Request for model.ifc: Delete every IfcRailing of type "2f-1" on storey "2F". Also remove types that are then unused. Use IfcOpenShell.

First a look at what the model holds.

```python
import ifcopenshell
import ifcopenshell.util.element

model = ifcopenshell.open("model.ifc")
print(model.schema)
storey = next(s for s in model.by_type("IfcBuildingStorey") if s.Name == "2F")
railings = [e for e in ifcopenshell.util.element.get_decomposition(storey) if e.is_a("IfcRailing")]
seen = {}
for e in railings:
    element_type = ifcopenshell.util.element.get_type(e)
    name = element_type.Name if element_type not in (None, e) else None
    seen[name] = seen.get(name, 0) + 1
for name, count in sorted(seen.items(), key=str):
    print(count, "x", name)
```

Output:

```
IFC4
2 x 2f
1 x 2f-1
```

```python
import ifcopenshell
import ifcopenshell.api.root
import ifcopenshell.util.element

model = ifcopenshell.open("model.ifc")

storey = next(s for s in model.by_type("IfcBuildingStorey") if s.Name == "2F")
railings = [e for e in ifcopenshell.util.element.get_decomposition(storey) if e.is_a("IfcRailing")]
targets = [e for e in railings if (t := ifcopenshell.util.element.get_type(e)) not in (None, e) and t.Name == "2f-1"]
types = {ifcopenshell.util.element.get_type(e) for e in targets} - {None, *targets}

for e in targets:
    ifcopenshell.api.root.remove_product(model, product=e)
print(len(targets), "removed")

unused = [t for t in types if not ifcopenshell.util.element.get_types(t)]
for t in unused:
    ifcopenshell.api.root.remove_product(model, product=t)
print(len(unused), "unused types removed")

model.write("model-out.ifc")
```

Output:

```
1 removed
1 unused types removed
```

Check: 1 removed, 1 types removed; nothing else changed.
